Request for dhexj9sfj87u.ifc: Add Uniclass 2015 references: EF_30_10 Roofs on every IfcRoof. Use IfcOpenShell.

First a look at what the model holds.

```python
import ifcopenshell

model = ifcopenshell.open("dhexj9sfj87u.ifc")
print(model.schema)
print("classifications:", [c.Name for c in model.by_type("IfcClassification")])
for ifc_class in ("IfcDoor", "IfcRoof", "IfcStair", "IfcWall", "IfcWindow"):
    print(ifc_class, len(model.by_type(ifc_class)))
```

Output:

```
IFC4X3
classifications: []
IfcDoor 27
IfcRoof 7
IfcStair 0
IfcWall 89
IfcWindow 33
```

```python
import ifcopenshell
import ifcopenshell.api.classification

model = ifcopenshell.open("dhexj9sfj87u.ifc")

system = ifcopenshell.api.classification.add_classification(model, classification="Uniclass 2015")

codes = {
    "IfcRoof": ("EF_30_10", "Roofs"),
}
for ifc_class, (code, name) in codes.items():
    products = model.by_type(ifc_class)
    ifcopenshell.api.classification.add_reference(
        model, products=products, classification=system, identification=code, name=name
    )
    print(code, len(products))

model.write("dhexj9sfj87u-out.ifc")
```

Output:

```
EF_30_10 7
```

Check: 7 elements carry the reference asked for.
